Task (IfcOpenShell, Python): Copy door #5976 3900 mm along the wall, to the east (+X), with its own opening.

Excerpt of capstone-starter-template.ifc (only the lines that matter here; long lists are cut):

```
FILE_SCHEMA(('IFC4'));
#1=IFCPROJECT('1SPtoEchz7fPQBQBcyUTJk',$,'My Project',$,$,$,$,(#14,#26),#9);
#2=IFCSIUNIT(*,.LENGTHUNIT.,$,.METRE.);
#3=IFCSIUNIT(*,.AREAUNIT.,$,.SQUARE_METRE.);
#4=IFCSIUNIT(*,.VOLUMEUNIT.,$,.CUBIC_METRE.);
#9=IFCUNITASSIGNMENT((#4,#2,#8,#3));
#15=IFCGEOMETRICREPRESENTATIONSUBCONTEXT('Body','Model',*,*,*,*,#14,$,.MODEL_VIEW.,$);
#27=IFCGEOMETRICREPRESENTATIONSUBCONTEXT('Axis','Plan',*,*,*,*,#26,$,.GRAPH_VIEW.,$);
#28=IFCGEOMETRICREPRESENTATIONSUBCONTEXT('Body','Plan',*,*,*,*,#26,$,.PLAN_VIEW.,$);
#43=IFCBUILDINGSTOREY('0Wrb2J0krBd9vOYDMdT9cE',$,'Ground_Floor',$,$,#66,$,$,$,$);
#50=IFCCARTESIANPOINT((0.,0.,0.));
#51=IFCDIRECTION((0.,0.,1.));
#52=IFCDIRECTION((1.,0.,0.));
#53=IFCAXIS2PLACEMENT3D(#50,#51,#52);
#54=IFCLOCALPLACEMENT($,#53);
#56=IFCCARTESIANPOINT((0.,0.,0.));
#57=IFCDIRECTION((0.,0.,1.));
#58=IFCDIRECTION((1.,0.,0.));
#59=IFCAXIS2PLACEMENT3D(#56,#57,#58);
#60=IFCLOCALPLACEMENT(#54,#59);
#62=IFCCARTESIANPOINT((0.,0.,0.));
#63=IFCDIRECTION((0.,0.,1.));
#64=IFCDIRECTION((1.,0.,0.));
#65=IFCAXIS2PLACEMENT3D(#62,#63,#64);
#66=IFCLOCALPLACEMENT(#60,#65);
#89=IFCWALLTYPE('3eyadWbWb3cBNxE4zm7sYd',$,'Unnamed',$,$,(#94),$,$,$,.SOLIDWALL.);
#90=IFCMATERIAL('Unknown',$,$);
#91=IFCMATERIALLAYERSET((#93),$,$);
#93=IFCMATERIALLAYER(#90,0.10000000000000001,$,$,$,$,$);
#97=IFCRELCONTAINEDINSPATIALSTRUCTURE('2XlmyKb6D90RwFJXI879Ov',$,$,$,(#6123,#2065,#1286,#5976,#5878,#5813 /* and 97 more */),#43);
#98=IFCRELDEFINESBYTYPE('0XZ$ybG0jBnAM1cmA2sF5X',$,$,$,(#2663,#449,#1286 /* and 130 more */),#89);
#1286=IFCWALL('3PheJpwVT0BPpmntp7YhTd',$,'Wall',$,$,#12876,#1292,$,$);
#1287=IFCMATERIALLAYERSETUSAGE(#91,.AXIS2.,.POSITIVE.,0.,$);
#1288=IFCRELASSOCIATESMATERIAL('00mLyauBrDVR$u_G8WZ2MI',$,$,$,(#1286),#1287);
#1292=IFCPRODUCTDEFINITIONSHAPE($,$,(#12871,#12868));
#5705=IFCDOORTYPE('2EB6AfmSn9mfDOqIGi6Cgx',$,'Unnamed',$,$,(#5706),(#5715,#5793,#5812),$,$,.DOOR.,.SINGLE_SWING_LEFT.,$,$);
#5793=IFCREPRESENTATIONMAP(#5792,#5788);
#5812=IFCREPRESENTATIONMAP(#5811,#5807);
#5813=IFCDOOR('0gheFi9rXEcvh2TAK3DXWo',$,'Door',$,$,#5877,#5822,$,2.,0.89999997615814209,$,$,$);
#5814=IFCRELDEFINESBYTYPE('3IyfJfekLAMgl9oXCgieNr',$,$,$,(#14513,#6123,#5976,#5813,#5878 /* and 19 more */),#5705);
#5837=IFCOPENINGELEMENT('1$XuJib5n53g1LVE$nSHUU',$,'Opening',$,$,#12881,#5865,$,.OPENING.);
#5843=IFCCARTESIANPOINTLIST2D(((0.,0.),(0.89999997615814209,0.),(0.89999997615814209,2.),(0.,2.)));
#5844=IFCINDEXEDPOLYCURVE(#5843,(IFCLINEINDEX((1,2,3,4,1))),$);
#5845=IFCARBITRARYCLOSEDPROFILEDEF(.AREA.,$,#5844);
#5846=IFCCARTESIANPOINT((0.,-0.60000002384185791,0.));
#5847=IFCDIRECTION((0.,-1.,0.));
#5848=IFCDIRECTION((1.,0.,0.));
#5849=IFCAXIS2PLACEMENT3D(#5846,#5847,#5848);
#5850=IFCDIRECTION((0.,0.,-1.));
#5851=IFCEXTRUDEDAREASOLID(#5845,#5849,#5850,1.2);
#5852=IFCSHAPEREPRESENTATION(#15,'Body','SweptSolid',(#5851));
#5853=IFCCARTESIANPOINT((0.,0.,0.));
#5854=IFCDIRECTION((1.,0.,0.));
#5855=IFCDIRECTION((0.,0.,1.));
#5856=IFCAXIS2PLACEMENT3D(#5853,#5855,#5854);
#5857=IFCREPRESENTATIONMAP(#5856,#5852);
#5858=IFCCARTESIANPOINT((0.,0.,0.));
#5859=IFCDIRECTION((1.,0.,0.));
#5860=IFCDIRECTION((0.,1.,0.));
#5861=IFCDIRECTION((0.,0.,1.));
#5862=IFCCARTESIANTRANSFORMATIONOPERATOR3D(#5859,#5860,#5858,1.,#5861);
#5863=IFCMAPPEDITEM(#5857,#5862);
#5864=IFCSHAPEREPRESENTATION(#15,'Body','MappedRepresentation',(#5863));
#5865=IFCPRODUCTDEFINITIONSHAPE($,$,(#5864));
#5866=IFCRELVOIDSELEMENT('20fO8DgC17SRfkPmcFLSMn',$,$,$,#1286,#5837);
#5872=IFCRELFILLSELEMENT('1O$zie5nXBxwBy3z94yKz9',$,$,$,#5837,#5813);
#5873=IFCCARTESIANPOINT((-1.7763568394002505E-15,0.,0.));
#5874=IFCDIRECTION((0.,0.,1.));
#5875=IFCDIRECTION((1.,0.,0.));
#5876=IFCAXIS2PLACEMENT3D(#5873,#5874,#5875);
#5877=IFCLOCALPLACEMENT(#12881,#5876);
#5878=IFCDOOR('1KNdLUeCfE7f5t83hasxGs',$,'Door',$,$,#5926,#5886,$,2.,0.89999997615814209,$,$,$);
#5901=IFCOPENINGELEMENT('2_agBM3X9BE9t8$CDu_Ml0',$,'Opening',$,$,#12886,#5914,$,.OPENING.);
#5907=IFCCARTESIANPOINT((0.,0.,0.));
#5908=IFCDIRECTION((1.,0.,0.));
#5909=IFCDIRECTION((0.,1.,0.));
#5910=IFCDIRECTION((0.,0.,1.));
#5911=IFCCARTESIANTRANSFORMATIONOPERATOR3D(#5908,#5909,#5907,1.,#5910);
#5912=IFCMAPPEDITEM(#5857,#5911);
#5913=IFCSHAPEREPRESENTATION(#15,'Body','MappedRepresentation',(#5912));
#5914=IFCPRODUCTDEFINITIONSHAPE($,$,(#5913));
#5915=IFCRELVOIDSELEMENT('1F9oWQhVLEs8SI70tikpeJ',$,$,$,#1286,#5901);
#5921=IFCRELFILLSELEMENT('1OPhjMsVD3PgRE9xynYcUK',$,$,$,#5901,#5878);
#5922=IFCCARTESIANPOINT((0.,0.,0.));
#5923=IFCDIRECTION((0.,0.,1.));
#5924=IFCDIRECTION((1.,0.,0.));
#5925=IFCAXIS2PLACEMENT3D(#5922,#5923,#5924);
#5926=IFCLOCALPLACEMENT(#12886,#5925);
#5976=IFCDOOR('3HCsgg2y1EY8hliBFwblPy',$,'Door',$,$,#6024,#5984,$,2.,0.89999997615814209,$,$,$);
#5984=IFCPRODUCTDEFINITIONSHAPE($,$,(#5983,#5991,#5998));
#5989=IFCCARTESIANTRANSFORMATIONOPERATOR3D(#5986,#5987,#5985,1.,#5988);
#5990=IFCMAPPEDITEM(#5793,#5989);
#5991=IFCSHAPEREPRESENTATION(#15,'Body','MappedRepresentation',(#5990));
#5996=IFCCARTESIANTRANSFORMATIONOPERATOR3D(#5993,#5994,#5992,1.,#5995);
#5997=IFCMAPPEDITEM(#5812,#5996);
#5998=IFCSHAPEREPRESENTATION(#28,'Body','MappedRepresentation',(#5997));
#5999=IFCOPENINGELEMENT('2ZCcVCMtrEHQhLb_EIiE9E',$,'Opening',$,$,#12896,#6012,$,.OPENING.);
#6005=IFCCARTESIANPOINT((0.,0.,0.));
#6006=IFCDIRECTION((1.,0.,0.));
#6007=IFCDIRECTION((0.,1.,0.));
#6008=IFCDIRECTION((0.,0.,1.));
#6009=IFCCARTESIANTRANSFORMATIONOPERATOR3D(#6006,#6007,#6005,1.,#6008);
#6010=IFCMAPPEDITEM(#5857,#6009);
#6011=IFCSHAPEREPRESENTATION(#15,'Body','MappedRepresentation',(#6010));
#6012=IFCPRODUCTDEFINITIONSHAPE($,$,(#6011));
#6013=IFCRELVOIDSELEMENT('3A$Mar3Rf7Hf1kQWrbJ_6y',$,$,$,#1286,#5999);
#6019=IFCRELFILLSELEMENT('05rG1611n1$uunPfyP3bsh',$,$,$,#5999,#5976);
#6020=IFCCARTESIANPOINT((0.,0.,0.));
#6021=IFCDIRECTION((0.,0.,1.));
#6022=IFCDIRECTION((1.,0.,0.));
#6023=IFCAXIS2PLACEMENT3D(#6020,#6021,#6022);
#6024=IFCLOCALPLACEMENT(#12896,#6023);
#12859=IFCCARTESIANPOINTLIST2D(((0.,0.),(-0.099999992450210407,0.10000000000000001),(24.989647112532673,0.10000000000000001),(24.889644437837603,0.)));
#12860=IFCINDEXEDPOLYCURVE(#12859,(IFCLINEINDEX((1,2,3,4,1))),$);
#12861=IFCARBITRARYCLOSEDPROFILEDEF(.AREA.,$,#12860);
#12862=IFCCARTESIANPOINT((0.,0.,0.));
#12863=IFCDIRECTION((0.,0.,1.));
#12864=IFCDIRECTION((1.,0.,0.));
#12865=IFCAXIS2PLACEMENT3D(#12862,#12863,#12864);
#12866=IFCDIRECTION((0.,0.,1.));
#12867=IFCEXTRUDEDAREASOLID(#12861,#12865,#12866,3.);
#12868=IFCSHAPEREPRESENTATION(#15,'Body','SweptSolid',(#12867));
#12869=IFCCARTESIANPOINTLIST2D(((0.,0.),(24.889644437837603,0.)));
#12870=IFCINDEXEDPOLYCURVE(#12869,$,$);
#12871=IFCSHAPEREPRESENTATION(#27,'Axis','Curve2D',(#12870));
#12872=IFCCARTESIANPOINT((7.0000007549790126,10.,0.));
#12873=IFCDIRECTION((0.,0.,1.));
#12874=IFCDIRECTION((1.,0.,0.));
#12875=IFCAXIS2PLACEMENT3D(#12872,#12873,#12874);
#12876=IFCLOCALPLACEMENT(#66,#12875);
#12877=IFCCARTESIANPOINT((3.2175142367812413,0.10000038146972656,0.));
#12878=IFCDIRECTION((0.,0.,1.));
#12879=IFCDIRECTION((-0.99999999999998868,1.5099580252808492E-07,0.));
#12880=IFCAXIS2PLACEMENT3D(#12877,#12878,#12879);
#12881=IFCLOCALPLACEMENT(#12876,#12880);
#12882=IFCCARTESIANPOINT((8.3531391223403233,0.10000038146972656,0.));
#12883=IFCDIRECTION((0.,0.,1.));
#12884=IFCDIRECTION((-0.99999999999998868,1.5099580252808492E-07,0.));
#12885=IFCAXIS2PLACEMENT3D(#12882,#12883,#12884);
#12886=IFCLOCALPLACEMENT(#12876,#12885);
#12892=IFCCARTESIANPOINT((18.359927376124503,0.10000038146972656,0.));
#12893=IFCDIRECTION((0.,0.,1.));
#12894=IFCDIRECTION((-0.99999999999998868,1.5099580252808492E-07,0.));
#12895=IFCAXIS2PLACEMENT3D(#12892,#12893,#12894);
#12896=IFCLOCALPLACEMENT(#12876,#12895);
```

```python
import ifcopenshell
import ifcopenshell.api.feature
import ifcopenshell.api.geometry
import ifcopenshell.api.root
import ifcopenshell.geom
import ifcopenshell.util.element
import ifcopenshell.util.placement
import ifcopenshell.util.shape

model = ifcopenshell.open("capstone-starter-template.ifc")
settings = ifcopenshell.geom.settings()


def volume(element):
    """Net volume in cubic metres, openings subtracted."""
    shape = ifcopenshell.geom.create_shape(settings, element)
    return ifcopenshell.util.shape.get_volume(shape.geometry)


door = model.by_guid("3HCsgg2y1EY8hliBFwblPy")
opening = door.FillsVoids[0].RelatingOpeningElement
wall = opening.VoidsElements[0].RelatingBuildingElement
before = volume(wall)
shift = ifcopenshell.util.placement.get_local_placement(wall.ObjectPlacement)[:3, 0] * 3.9

# copy_class copies the void relationship, type, container and properties, but no geometry.
new_opening = ifcopenshell.api.root.copy_class(model, product=opening)
new_opening.Representation = ifcopenshell.util.element.copy_deep(
    model, opening.Representation, exclude=["IfcGeometricRepresentationContext", "IfcRepresentationMap"]
)
new_door = ifcopenshell.api.root.copy_class(model, product=door)
new_door.Representation = ifcopenshell.util.element.copy_deep(
    model, door.Representation, exclude=["IfcGeometricRepresentationContext", "IfcRepresentationMap"]
)
ifcopenshell.api.feature.add_filling(model, opening=new_opening, element=new_door)

for old, new in ((opening, new_opening), (door, new_door)):
    matrix = ifcopenshell.util.placement.get_local_placement(old.ObjectPlacement)
    matrix[:3, 3] += shift
    ifcopenshell.api.geometry.edit_object_placement(model, product=new, matrix=matrix, is_si=False)

after = volume(wall)

print(f"wall volume {before:.3f} -> {after:.3f} m3")

model.write("capstone-starter-template_edited.ifc")
```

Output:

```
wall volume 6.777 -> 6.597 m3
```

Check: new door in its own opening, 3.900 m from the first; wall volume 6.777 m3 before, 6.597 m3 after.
